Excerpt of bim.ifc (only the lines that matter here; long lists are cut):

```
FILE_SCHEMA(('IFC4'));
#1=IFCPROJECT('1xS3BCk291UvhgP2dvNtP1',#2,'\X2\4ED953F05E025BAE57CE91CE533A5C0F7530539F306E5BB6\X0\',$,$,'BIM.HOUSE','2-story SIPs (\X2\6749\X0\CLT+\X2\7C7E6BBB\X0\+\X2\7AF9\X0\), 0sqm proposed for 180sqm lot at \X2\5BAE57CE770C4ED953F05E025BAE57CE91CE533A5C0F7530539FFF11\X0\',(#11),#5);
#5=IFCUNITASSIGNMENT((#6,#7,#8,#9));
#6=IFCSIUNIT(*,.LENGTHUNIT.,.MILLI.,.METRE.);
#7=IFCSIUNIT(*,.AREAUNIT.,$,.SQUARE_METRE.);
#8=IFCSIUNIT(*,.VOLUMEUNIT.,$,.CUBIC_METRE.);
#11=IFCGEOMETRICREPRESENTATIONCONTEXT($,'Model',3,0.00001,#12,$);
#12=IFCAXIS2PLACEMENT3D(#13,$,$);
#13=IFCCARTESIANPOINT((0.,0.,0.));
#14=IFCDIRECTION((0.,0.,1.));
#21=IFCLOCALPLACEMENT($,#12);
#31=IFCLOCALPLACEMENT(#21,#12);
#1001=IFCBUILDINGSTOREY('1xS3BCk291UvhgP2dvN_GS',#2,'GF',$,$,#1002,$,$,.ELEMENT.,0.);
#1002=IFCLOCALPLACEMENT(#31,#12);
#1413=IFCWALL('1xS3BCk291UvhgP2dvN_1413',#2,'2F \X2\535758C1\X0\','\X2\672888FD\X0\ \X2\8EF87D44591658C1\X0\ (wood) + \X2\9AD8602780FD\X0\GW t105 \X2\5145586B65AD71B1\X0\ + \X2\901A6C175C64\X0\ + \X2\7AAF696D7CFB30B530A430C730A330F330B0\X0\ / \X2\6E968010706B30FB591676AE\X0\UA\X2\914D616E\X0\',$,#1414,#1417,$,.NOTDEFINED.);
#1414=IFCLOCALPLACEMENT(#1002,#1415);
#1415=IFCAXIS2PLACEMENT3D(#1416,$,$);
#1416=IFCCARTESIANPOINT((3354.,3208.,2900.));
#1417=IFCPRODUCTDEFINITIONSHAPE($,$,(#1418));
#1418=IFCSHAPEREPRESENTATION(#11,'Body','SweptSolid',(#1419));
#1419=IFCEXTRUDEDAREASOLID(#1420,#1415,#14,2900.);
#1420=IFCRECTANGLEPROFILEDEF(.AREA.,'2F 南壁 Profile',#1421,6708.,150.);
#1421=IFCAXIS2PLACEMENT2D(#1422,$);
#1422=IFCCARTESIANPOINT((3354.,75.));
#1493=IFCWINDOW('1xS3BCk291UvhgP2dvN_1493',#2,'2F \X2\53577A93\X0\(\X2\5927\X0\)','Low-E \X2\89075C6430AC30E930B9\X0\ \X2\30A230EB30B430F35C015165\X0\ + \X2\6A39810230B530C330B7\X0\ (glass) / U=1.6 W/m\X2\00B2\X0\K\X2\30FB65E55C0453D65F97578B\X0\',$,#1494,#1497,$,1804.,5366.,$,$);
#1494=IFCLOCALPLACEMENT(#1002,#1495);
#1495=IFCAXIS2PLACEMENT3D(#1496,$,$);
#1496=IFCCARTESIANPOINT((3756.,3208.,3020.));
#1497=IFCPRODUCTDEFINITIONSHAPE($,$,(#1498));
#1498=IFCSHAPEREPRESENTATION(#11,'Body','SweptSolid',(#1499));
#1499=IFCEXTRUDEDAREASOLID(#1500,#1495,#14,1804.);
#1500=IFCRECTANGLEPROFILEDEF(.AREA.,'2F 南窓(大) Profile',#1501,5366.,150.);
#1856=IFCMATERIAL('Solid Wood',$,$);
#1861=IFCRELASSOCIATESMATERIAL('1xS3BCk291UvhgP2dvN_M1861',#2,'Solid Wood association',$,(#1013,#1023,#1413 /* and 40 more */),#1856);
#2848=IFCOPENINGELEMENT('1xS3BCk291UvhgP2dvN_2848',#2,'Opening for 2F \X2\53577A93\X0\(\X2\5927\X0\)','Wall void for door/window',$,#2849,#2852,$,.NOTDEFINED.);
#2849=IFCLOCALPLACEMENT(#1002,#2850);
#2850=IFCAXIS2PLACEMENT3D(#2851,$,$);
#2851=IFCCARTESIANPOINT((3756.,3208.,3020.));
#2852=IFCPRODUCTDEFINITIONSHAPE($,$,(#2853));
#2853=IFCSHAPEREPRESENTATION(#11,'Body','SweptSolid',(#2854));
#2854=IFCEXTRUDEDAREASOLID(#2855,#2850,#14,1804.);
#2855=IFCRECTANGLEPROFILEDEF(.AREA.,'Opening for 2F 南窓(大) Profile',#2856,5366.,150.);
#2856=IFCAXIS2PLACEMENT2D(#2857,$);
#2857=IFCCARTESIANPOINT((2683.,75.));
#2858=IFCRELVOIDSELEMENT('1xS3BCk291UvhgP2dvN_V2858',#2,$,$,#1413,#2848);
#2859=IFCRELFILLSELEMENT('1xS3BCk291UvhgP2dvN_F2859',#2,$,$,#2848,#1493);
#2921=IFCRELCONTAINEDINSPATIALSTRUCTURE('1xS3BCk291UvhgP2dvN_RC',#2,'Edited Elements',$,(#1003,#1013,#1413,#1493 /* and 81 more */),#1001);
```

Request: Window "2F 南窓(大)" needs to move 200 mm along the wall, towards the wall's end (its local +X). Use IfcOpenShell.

```python
import ifcopenshell
import ifcopenshell.api.geometry
import ifcopenshell.util.placement
import ifcopenshell.util.unit

model = ifcopenshell.open("bim.ifc")
unit_scale = ifcopenshell.util.unit.calculate_unit_scale(model)

window = model.by_guid("1xS3BCk291UvhgP2dvN_1493")
opening = window.FillsVoids[0].RelatingOpeningElement
wall = opening.VoidsElements[0].RelatingBuildingElement

wall_matrix = ifcopenshell.util.placement.get_local_placement(wall.ObjectPlacement)
shift = wall_matrix[:3, 0] * 0.2 / unit_scale
before = ifcopenshell.util.placement.get_local_placement(window.ObjectPlacement)[:3, 3].copy()

# The window is not placed relative to its opening, so move both.
for product in (opening, window):
    matrix = ifcopenshell.util.placement.get_local_placement(product.ObjectPlacement)
    matrix[:3, 3] += shift
    ifcopenshell.api.geometry.edit_object_placement(model, product=product, matrix=matrix, is_si=False)

after = ifcopenshell.util.placement.get_local_placement(window.ObjectPlacement)[:3, 3]
print("window moved by", (after - before).round(3) + 0.0)

model.write("bim_updated.ifc")
```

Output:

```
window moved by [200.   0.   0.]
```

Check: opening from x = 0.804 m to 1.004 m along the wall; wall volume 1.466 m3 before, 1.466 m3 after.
